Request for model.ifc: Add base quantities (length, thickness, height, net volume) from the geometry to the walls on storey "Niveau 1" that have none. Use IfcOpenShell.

First a look at what the model holds.

```python
import ifcopenshell
import ifcopenshell.util.element
import ifcopenshell.util.unit

model = ifcopenshell.open("model.ifc")
print(model.schema)
for unit_type in ("LENGTHUNIT", "AREAUNIT", "VOLUMEUNIT"):
    print(unit_type, ifcopenshell.util.unit.calculate_unit_scale(model, unit_type))
storey = next(s for s in model.by_type("IfcBuildingStorey") if s.Name == "Niveau 1")
walls = [e for e in ifcopenshell.util.element.get_decomposition(storey) if e.is_a("IfcWall")]
for e in sorted(walls, key=lambda e: e.id()):
    print(e.id(), e.is_a(), e.Name, list(ifcopenshell.util.element.get_psets(e, qtos_only=True)), sep=" | ")
```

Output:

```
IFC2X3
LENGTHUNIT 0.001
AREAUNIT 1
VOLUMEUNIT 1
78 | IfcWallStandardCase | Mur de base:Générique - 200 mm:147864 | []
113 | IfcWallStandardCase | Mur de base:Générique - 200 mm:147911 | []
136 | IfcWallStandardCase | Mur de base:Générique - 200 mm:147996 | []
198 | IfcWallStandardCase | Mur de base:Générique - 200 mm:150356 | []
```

```python
import ifcopenshell
import ifcopenshell.api.pset
import ifcopenshell.geom
import ifcopenshell.util.element
import ifcopenshell.util.shape
import ifcopenshell.util.unit

model = ifcopenshell.open("model.ifc")
unit_scale = ifcopenshell.util.unit.calculate_unit_scale(model)
volume_scale = ifcopenshell.util.unit.calculate_unit_scale(model, "VOLUMEUNIT")
settings = ifcopenshell.geom.settings()

storey = next(s for s in model.by_type("IfcBuildingStorey") if s.Name == "Niveau 1")
walls = [e for e in ifcopenshell.util.element.get_decomposition(storey) if e.is_a("IfcWall")]

for e in sorted(walls, key=lambda e: e.id()):
    if ifcopenshell.util.element.get_psets(e, qtos_only=True, should_inherit=False):
        continue
    # Geometry comes back in metres, in the element's own axes.
    shape = ifcopenshell.geom.create_shape(settings, e)
    values = {
        "Length": ifcopenshell.util.shape.get_x(shape.geometry) / unit_scale,
        "Width": ifcopenshell.util.shape.get_y(shape.geometry) / unit_scale,
        "Height": ifcopenshell.util.shape.get_z(shape.geometry) / unit_scale,
        "NetVolume": ifcopenshell.util.shape.get_volume(shape.geometry) / volume_scale,
    }
    qto = ifcopenshell.api.pset.add_qto(model, product=e, name="BaseQuantities")
    ifcopenshell.api.pset.edit_qto(model, qto=qto, properties=values)
    print(e.id(), {k: round(v, 3) for k, v in values.items()})

model.write("model-out.ifc")
```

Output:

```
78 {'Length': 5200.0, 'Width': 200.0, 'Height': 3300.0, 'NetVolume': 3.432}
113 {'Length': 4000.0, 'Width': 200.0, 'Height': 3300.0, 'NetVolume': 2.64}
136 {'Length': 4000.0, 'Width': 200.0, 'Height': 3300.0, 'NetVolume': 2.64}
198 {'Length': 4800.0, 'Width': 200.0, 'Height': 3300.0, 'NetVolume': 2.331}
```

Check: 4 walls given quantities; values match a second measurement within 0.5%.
